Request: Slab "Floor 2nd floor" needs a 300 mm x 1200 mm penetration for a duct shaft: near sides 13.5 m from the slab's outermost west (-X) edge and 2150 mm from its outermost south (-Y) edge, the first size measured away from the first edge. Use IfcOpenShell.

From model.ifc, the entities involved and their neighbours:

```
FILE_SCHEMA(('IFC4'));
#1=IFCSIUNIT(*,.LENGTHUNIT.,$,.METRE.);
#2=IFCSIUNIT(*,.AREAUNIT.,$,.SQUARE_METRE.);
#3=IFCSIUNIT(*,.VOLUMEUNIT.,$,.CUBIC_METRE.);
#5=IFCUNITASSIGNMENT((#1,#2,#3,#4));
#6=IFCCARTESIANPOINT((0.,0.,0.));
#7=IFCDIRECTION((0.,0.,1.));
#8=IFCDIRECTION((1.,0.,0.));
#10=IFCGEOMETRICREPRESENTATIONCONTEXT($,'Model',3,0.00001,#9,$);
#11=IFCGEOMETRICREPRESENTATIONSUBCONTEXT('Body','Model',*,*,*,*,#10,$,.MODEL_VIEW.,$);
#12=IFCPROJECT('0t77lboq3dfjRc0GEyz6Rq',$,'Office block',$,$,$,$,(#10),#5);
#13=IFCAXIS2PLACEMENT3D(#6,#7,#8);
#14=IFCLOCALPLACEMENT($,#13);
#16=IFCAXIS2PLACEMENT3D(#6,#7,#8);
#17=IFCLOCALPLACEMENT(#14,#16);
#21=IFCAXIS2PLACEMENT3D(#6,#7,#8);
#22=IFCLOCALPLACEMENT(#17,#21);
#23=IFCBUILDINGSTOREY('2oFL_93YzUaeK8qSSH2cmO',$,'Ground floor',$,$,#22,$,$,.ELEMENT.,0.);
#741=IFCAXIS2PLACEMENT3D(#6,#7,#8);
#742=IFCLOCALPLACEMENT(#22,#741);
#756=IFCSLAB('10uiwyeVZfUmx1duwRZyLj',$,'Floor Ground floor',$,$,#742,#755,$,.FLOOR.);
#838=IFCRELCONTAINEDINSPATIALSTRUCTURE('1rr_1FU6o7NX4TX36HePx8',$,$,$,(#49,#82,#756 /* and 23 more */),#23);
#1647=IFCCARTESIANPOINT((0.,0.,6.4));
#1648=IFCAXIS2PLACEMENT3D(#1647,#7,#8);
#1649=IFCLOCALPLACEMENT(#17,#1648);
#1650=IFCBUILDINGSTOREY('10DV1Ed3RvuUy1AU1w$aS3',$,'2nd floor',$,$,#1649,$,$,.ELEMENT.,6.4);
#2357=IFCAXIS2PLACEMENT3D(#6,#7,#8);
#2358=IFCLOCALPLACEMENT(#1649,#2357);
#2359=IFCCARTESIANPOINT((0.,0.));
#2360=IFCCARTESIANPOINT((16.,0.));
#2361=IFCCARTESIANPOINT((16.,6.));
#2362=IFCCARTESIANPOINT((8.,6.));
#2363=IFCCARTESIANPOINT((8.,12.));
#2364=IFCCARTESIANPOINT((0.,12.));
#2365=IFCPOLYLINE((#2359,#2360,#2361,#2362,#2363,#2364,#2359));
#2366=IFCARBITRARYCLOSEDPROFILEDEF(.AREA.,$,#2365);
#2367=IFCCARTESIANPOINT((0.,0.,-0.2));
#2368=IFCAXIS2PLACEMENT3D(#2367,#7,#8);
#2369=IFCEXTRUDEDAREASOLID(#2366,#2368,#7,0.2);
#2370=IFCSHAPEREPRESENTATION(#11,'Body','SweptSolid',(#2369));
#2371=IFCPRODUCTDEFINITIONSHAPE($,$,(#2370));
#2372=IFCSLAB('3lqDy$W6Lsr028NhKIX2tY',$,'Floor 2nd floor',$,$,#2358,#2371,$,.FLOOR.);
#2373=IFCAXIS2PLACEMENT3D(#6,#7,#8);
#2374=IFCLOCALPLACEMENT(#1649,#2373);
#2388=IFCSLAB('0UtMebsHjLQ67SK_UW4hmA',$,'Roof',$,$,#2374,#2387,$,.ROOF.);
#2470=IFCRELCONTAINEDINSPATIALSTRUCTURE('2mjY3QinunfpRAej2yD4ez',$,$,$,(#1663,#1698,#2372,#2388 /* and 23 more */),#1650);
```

```python
import numpy as np
import ifcopenshell
import ifcopenshell.api.feature
import ifcopenshell.api.geometry
import ifcopenshell.api.root
import ifcopenshell.geom
import ifcopenshell.util.placement
import ifcopenshell.util.representation
import ifcopenshell.util.shape
import ifcopenshell.util.unit

model = ifcopenshell.open("model.ifc")
unit_scale = ifcopenshell.util.unit.calculate_unit_scale(model)
settings = ifcopenshell.geom.settings()


def volume(element):
    """Net volume in cubic metres, openings subtracted."""
    shape = ifcopenshell.geom.create_shape(settings, element)
    return ifcopenshell.util.shape.get_volume(shape.geometry)


slab = model.by_guid("3lqDy$W6Lsr028NhKIX2tY")
before = volume(slab)

# Extent in the slab's own axes, in metres. The edges named are its -X and -Y sides.
slab_shape = ifcopenshell.geom.create_shape(settings, slab)
vertices = ifcopenshell.util.shape.get_vertices(slab_shape.geometry)
x_min, y_min, bottom = vertices.min(axis=0)
top = vertices[:, 2].max()

opening = ifcopenshell.api.root.create_entity(model, ifc_class="IfcOpeningElement", name="Duct shaft opening", predefined_type="OPENING")
context = ifcopenshell.util.representation.get_context(model, "Model", "Body", "MODEL_VIEW")
width, depth = 0.3, 1.2
outline = [(0.0, 0.0), (width, 0.0), (width, depth), (0.0, depth), (0.0, 0.0)]
# Overshoot both faces by 50 mm so the cut is clean.
shape = ifcopenshell.api.geometry.add_slab_representation(
    model, context=context, depth=top - bottom + 0.1, polyline=outline
)
ifcopenshell.api.geometry.assign_representation(model, product=opening, representation=shape)

matrix = ifcopenshell.util.placement.get_local_placement(slab.ObjectPlacement)
matrix[:, 3] = matrix @ np.append(np.array([x_min + 13.5, y_min + 2.15, bottom - 0.05]) / unit_scale, 1.0)
ifcopenshell.api.geometry.edit_object_placement(model, product=opening, matrix=matrix, is_si=False)
ifcopenshell.api.feature.add_feature(model, feature=opening, element=slab)

after = volume(slab)

print(f"slab volume {before:.3f} -> {after:.3f} m3")

model.write("model_edited.ifc")
```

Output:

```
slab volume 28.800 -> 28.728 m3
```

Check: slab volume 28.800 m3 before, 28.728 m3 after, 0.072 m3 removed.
